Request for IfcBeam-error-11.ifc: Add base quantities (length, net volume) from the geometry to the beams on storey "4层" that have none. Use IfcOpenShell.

First a look at what the model holds.

```python
import ifcopenshell
import ifcopenshell.util.element
import ifcopenshell.util.unit

model = ifcopenshell.open("IfcBeam-error-11.ifc")
print(model.schema)
for unit_type in ("LENGTHUNIT", "AREAUNIT", "VOLUMEUNIT"):
    print(unit_type, ifcopenshell.util.unit.calculate_unit_scale(model, unit_type))
storey = next(s for s in model.by_type("IfcBuildingStorey") if s.Name == "4层")
beams = [e for e in ifcopenshell.util.element.get_decomposition(storey) if e.is_a("IfcBeam")]
for e in sorted(beams, key=lambda e: e.id()):
    print(e.id(), e.is_a(), e.Name, list(ifcopenshell.util.element.get_psets(e, qtos_only=True)), sep=" | ")
```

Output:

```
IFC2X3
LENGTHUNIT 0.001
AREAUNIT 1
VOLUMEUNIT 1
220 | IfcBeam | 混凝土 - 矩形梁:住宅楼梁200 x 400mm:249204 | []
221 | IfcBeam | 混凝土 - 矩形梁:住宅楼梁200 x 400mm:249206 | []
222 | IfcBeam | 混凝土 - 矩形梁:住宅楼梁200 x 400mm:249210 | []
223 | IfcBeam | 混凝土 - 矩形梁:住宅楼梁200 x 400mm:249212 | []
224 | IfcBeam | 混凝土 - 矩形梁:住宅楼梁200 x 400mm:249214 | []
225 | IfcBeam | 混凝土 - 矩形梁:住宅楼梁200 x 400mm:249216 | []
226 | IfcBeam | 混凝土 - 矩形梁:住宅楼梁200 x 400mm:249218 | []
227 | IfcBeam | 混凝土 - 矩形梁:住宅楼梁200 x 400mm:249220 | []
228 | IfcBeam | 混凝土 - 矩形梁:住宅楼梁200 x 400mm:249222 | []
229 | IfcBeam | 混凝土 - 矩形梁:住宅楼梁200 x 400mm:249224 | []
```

```python
import ifcopenshell
import ifcopenshell.api.pset
import ifcopenshell.geom
import ifcopenshell.util.element
import ifcopenshell.util.shape
import ifcopenshell.util.unit

model = ifcopenshell.open("IfcBeam-error-11.ifc")
unit_scale = ifcopenshell.util.unit.calculate_unit_scale(model)
volume_scale = ifcopenshell.util.unit.calculate_unit_scale(model, "VOLUMEUNIT")
settings = ifcopenshell.geom.settings()

storey = next(s for s in model.by_type("IfcBuildingStorey") if s.Name == "4层")
beams = [e for e in ifcopenshell.util.element.get_decomposition(storey) if e.is_a("IfcBeam")]

for e in sorted(beams, key=lambda e: e.id()):
    if ifcopenshell.util.element.get_psets(e, qtos_only=True, should_inherit=False):
        continue
    # Geometry comes back in metres, in the element's own axes.
    shape = ifcopenshell.geom.create_shape(settings, e)
    values = {
        "Length": ifcopenshell.util.shape.get_max_xyz(shape.geometry) / unit_scale,
        "NetVolume": ifcopenshell.util.shape.get_volume(shape.geometry) / volume_scale,
    }
    qto = ifcopenshell.api.pset.add_qto(model, product=e, name="BaseQuantities")
    ifcopenshell.api.pset.edit_qto(model, qto=qto, properties=values)
    print(e.id(), {k: round(v, 3) for k, v in values.items()})

model.write("IfcBeam-error-11_rev.ifc")
```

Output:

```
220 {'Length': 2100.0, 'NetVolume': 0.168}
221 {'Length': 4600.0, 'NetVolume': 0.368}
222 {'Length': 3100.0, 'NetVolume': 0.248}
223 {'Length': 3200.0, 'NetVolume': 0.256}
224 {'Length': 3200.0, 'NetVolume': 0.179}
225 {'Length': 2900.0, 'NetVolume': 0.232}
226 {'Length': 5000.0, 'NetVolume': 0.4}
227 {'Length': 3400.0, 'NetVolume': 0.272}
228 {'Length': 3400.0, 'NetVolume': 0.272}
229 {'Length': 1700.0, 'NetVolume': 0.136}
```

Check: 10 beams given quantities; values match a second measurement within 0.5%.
